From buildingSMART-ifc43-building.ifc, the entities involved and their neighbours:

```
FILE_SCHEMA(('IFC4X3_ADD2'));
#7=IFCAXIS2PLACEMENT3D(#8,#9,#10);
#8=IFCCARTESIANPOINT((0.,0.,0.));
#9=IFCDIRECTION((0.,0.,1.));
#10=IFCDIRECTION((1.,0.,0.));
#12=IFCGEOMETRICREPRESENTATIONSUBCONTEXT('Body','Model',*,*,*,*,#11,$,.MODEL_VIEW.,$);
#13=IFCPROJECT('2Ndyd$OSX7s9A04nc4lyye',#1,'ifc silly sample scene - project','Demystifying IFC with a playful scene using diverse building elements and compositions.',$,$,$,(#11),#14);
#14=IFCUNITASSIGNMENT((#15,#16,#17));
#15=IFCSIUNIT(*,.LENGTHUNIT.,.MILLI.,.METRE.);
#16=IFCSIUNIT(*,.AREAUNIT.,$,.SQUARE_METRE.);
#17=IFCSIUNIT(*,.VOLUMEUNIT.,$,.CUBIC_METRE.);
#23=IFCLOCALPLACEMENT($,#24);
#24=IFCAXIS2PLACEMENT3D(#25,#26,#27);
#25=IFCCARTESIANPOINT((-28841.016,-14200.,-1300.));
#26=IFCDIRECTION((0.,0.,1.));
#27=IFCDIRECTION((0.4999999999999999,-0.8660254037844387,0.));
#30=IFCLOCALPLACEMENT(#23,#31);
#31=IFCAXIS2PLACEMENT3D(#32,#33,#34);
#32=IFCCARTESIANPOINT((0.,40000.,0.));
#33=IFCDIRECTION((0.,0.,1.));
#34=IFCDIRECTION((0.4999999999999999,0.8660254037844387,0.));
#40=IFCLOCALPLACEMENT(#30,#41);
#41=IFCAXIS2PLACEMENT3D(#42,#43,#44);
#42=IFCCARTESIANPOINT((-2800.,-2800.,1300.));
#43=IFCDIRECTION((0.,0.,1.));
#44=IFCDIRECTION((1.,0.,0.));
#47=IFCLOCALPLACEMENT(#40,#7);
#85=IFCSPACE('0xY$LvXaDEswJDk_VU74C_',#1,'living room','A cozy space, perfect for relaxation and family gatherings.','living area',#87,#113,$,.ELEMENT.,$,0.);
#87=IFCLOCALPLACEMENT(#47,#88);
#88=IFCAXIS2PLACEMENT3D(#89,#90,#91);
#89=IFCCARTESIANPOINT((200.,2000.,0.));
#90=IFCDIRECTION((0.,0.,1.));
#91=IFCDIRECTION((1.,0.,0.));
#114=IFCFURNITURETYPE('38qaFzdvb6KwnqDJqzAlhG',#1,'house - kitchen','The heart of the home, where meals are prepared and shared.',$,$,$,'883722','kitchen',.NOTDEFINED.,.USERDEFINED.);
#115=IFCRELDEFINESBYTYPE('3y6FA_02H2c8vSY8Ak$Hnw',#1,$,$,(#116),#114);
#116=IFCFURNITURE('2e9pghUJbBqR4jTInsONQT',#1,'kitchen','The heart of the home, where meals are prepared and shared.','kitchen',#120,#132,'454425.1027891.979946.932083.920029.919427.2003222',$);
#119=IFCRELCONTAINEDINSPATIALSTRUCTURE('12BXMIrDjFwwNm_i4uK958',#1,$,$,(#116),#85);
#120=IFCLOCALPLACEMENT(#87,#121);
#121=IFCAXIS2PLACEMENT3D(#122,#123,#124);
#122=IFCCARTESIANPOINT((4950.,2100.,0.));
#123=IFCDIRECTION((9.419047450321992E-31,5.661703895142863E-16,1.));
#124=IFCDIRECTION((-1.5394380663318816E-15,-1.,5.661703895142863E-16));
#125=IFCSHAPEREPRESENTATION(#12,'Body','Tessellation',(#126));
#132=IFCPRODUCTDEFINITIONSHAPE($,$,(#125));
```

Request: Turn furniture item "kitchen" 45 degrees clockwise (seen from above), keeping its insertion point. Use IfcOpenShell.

```python
import ifcopenshell
import ifcopenshell.api.geometry
import ifcopenshell.util.placement

model = ifcopenshell.open("buildingSMART-ifc43-building.ifc")

item = model.by_guid("2e9pghUJbBqR4jTInsONQT")
matrix = ifcopenshell.util.placement.get_local_placement(item.ObjectPlacement)
matrix = matrix @ ifcopenshell.util.placement.rotation(-45, "Z")
ifcopenshell.api.geometry.edit_object_placement(model, product=item, matrix=matrix, is_si=False)

print(ifcopenshell.util.placement.get_local_placement(item.ObjectPlacement).round(3) + 0.0)

model.write("buildingSMART-ifc43-building_rev.ifc")
```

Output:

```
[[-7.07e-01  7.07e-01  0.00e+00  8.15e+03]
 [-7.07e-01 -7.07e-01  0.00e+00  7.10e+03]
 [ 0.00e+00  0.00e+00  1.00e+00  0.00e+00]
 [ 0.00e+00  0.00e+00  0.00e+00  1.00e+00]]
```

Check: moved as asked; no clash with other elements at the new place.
